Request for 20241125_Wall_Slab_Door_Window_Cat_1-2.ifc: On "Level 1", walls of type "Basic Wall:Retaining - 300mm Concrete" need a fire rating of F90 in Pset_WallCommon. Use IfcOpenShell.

First a look at what the model holds.

```python
import ifcopenshell
import ifcopenshell.util.element

model = ifcopenshell.open("20241125_Wall_Slab_Door_Window_Cat_1-2.ifc")
print(model.schema)
storey = next(s for s in model.by_type("IfcBuildingStorey") if s.Name == "Level 1")
walls = [e for e in ifcopenshell.util.element.get_decomposition(storey) if e.is_a("IfcWall")]
seen = {}
for e in walls:
    element_type = ifcopenshell.util.element.get_type(e)
    key = (element_type.Name if element_type != e and element_type else None, ifcopenshell.util.element.get_pset(e, "Pset_WallCommon", "FireRating"))
    seen[key] = seen.get(key, 0) + 1
for (name, value), count in sorted(seen.items(), key=str):
    print(count, "x", name, "|", value)
```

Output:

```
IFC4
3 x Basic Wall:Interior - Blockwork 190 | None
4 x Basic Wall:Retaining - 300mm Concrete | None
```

```python
import ifcopenshell
import ifcopenshell.api.pset
import ifcopenshell.util.element

model = ifcopenshell.open("20241125_Wall_Slab_Door_Window_Cat_1-2.ifc")

storey = next(s for s in model.by_type("IfcBuildingStorey") if s.Name == "Level 1")
walls = [e for e in ifcopenshell.util.element.get_decomposition(storey) if e.is_a("IfcWall")]

count = 0
for e in walls:
    element_type = ifcopenshell.util.element.get_type(e)
    if element_type in (None, e) or element_type.Name != "Basic Wall:Retaining - 300mm Concrete":
        continue
    # add_pset returns the element's existing set when there is one.
    pset = ifcopenshell.api.pset.add_pset(model, product=e, name="Pset_WallCommon")
    ifcopenshell.api.pset.edit_pset(model, pset=pset, properties={"FireRating": "F90"})
    count += 1

print(count, "walls updated")

model.write("20241125_Wall_Slab_Door_Window_Cat_1-2-out.ifc")
```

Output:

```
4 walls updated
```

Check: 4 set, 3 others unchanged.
